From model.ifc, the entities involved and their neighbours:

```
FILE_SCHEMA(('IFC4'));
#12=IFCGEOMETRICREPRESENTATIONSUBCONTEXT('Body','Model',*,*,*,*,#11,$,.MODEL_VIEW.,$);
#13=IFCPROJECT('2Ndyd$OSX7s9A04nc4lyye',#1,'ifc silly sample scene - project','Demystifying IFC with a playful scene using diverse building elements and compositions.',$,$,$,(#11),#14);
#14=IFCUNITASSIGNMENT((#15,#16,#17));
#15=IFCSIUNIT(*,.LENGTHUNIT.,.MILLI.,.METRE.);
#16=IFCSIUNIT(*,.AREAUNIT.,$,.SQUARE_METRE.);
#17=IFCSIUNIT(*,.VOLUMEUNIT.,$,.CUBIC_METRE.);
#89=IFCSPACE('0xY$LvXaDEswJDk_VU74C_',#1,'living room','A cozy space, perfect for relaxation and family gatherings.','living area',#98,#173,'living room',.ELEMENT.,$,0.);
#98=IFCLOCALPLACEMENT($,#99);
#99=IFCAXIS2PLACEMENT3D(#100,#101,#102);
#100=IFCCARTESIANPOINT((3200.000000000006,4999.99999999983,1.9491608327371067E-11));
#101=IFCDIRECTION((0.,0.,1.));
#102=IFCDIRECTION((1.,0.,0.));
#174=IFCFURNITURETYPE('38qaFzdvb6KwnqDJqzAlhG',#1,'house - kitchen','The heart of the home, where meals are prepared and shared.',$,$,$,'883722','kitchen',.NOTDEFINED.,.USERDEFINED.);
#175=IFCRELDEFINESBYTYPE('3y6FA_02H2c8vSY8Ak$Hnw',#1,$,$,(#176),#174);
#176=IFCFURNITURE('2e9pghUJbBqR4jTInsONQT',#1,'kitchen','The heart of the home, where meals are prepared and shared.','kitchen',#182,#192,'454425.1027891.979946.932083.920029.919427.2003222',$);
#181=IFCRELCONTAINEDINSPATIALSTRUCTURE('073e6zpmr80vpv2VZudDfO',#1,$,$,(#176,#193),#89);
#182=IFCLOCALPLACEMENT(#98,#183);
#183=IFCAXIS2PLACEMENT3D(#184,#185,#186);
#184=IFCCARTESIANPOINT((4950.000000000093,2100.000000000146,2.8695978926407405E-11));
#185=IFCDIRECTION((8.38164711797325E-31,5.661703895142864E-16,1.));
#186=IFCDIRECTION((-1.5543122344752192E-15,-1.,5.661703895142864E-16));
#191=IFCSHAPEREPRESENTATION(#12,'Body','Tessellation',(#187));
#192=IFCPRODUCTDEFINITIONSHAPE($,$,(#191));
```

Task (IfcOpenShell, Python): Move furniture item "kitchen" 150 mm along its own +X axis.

```python
import ifcopenshell
import ifcopenshell.api.geometry
import ifcopenshell.util.placement
import ifcopenshell.util.unit

model = ifcopenshell.open("model.ifc")
unit_scale = ifcopenshell.util.unit.calculate_unit_scale(model)

item = model.by_id(176)
matrix = ifcopenshell.util.placement.get_local_placement(item.ObjectPlacement)
matrix[:3, 3] += matrix[:3, 0] * 0.15 / unit_scale
ifcopenshell.api.geometry.edit_object_placement(model, product=item, matrix=matrix, is_si=False)

print(ifcopenshell.util.placement.get_local_placement(item.ObjectPlacement).round(3) + 0.0)

model.write("model_edited.ifc")
```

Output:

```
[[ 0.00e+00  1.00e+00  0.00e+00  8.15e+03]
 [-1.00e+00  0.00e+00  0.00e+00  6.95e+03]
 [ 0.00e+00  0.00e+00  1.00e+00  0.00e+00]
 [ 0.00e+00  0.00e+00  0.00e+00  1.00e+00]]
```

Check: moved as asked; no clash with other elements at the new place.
